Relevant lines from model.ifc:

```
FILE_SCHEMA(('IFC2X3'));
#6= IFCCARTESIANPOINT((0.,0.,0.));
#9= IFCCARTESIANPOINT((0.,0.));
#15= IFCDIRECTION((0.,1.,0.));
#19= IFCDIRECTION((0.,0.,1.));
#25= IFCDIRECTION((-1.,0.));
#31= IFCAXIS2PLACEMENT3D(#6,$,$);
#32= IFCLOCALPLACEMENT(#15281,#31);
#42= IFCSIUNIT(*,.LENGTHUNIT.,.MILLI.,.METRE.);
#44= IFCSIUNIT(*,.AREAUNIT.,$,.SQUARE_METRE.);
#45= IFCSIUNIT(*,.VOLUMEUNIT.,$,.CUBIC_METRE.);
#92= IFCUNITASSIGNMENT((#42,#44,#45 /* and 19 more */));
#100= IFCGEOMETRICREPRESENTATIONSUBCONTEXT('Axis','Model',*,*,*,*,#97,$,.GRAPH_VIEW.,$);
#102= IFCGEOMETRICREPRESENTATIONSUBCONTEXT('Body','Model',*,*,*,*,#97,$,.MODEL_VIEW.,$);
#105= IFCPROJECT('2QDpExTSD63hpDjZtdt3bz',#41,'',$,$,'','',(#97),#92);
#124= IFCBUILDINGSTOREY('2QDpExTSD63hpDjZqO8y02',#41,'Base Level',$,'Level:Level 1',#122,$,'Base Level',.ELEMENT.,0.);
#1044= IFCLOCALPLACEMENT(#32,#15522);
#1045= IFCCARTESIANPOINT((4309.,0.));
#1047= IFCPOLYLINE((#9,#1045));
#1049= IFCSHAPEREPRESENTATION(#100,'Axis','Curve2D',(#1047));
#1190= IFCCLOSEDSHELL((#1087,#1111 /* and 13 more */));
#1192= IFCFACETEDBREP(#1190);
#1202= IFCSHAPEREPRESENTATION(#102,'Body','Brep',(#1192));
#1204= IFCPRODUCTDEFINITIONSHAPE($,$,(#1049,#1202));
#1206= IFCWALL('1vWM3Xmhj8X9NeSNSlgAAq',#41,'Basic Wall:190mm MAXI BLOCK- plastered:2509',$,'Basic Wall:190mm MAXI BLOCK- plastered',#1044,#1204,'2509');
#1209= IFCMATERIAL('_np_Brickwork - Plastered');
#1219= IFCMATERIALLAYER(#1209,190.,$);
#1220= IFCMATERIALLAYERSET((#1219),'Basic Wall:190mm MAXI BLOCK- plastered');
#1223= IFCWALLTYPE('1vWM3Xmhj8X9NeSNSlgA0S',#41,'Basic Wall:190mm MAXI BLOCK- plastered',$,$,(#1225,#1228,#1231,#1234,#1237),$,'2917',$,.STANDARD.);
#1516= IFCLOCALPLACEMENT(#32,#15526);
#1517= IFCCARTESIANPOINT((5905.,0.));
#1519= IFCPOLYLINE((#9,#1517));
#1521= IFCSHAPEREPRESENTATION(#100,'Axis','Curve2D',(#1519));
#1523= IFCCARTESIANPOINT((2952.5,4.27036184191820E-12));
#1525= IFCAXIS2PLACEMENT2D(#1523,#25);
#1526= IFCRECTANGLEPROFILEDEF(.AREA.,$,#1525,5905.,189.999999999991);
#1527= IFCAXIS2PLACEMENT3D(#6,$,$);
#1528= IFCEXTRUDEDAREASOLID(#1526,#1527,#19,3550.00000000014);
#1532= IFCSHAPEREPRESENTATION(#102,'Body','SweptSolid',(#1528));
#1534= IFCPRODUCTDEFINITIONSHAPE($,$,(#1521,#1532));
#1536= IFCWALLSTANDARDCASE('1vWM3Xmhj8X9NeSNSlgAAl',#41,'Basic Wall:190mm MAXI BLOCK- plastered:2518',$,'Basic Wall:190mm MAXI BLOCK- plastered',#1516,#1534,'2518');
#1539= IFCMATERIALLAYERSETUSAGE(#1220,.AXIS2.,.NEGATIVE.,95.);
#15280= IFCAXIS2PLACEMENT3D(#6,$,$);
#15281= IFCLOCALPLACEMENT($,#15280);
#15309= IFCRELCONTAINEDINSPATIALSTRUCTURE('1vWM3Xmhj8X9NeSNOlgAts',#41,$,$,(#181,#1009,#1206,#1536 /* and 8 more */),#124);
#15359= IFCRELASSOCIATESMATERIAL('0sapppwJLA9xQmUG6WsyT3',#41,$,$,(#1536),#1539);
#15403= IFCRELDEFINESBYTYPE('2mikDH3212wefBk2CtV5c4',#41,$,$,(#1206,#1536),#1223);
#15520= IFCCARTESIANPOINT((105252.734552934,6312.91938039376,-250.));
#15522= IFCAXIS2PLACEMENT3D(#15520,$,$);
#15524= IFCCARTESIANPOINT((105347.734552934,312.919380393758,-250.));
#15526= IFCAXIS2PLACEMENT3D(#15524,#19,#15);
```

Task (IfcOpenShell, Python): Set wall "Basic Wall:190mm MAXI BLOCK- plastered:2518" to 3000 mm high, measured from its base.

```python
import ifcopenshell
import ifcopenshell.geom
import ifcopenshell.util.representation
import ifcopenshell.util.shape

model = ifcopenshell.open("model.ifc")
settings = ifcopenshell.geom.settings()


def volume(element):
    """Net volume in cubic metres, openings subtracted."""
    shape = ifcopenshell.geom.create_shape(settings, element)
    return ifcopenshell.util.shape.get_volume(shape.geometry)


wall = model.by_guid("1vWM3Xmhj8X9NeSNSlgAAl")
before = volume(wall)

body = ifcopenshell.util.representation.get_representation(wall, "Model", "Body")
solid = body.Items[0]
old_height = solid.Depth
solid.Depth = 3000.0
after = volume(wall)

print(f"height {old_height:g} -> {solid.Depth:g}, volume {before:.3f} -> {after:.3f} m3")

model.write("model_updated.ifc")
```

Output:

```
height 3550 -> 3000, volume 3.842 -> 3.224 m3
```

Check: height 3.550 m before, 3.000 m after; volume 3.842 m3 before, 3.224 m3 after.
